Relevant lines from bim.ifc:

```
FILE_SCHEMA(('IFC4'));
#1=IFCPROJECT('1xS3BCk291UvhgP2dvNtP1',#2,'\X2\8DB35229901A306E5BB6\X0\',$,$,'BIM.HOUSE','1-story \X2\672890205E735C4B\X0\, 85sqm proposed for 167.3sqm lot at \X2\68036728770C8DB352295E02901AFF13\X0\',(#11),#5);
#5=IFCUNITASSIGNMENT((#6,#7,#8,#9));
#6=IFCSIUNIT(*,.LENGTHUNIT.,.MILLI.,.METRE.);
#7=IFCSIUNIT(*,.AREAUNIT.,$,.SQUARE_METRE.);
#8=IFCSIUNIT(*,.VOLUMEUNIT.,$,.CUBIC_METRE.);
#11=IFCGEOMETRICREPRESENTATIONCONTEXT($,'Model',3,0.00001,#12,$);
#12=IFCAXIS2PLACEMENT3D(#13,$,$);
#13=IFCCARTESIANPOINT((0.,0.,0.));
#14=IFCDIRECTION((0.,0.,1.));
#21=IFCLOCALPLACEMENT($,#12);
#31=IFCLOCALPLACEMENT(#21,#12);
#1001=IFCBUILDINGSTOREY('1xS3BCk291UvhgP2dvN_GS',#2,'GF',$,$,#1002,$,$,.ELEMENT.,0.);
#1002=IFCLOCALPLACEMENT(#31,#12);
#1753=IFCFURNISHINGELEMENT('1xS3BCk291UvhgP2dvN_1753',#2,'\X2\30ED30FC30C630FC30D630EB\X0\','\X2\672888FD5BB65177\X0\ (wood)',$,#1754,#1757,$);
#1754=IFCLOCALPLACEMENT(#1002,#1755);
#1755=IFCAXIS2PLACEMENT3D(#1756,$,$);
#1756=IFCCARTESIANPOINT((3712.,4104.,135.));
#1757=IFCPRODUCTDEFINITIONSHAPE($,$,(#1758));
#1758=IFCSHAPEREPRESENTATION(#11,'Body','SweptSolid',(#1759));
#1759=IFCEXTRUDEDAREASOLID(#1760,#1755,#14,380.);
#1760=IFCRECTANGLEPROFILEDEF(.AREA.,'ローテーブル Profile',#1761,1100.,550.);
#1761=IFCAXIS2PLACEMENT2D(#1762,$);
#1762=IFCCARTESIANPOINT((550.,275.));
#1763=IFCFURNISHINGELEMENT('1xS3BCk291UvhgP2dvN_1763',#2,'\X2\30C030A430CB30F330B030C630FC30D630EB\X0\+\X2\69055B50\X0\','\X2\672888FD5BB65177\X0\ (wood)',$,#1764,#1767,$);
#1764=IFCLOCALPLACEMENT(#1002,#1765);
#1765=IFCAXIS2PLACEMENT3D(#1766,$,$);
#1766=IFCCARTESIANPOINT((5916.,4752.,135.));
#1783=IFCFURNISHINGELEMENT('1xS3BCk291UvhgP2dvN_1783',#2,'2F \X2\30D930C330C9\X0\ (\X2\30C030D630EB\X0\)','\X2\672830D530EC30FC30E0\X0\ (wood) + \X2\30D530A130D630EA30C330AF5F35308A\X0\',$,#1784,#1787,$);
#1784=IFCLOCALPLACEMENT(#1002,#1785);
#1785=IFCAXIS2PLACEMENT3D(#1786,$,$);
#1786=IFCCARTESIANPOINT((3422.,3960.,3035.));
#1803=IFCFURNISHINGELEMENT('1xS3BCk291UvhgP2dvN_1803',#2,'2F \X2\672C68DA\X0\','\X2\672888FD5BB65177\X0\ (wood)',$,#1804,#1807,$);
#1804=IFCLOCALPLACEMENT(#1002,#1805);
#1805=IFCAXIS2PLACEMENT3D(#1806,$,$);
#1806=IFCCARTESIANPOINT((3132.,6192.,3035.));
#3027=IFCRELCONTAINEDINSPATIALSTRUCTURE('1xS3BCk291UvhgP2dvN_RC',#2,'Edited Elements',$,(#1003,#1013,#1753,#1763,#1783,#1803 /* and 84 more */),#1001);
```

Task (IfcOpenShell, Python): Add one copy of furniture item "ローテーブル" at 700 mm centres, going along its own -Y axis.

```python
import ifcopenshell
import ifcopenshell.api.geometry
import ifcopenshell.api.root
import ifcopenshell.util.element
import ifcopenshell.util.placement
import ifcopenshell.util.unit

model = ifcopenshell.open("bim.ifc")
unit_scale = ifcopenshell.util.unit.calculate_unit_scale(model)


def reuse_history(source, copy):
    """copy_class also copies each property set's owner history, people and application; keep the originals."""
    for rel in copy.IsDefinedBy:
        if rel.is_a("IfcRelDefinesByProperties") and (history := rel.RelatingPropertyDefinition.OwnerHistory):
            rel.RelatingPropertyDefinition.OwnerHistory = source.OwnerHistory
            ifcopenshell.util.element.remove_deep2(model, history)


source = model.by_guid("1xS3BCk291UvhgP2dvN_1753")
base = ifcopenshell.util.placement.get_local_placement(source.ObjectPlacement)
step = -base[:3, 1] * 0.7 / unit_scale

for i in range(1, 2):
    copy = ifcopenshell.api.root.copy_class(model, product=source)
    copy.Representation = ifcopenshell.util.element.copy_deep(
        model, source.Representation, exclude=["IfcGeometricRepresentationContext", "IfcRepresentationMap"]
    )
    reuse_history(source, copy)
    matrix = base.copy()
    matrix[:3, 3] += i * step
    print("added at", matrix[:3, 3].round(3) + 0.0)
    ifcopenshell.api.geometry.edit_object_placement(model, product=copy, matrix=matrix, is_si=False)

model.write("bim_edited.ifc")
```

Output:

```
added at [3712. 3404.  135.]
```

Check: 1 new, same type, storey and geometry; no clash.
